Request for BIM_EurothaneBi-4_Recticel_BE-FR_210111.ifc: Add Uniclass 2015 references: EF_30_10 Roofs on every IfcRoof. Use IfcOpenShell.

First a look at what the model holds.

```python
import ifcopenshell

model = ifcopenshell.open("BIM_EurothaneBi-4_Recticel_BE-FR_210111.ifc")
print(model.schema)
print("classifications:", [c.Name for c in model.by_type("IfcClassification")])
for ifc_class in ("IfcDoor", "IfcRoof", "IfcStair", "IfcWall", "IfcWindow"):
    print(ifc_class, len(model.by_type(ifc_class)))
```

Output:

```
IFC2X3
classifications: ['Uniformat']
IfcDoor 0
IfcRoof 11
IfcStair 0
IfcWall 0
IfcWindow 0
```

```python
import ifcopenshell
import ifcopenshell.api.classification

model = ifcopenshell.open("BIM_EurothaneBi-4_Recticel_BE-FR_210111.ifc")

# IFC2X3 requires Source and Edition and has no link from the project to the system.
system = model.create_entity("IfcClassification", Source="NBS", Edition="2015", Name="Uniclass 2015")

codes = {
    "IfcRoof": ("EF_30_10", "Roofs"),
}
for ifc_class, (code, name) in codes.items():
    products = model.by_type(ifc_class)
    ifcopenshell.api.classification.add_reference(
        model, products=products, classification=system, identification=code, name=name
    )
    print(code, len(products))

model.write("BIM_EurothaneBi-4_Recticel_BE-FR_210111_rev.ifc")
```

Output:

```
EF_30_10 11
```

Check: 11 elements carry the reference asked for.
